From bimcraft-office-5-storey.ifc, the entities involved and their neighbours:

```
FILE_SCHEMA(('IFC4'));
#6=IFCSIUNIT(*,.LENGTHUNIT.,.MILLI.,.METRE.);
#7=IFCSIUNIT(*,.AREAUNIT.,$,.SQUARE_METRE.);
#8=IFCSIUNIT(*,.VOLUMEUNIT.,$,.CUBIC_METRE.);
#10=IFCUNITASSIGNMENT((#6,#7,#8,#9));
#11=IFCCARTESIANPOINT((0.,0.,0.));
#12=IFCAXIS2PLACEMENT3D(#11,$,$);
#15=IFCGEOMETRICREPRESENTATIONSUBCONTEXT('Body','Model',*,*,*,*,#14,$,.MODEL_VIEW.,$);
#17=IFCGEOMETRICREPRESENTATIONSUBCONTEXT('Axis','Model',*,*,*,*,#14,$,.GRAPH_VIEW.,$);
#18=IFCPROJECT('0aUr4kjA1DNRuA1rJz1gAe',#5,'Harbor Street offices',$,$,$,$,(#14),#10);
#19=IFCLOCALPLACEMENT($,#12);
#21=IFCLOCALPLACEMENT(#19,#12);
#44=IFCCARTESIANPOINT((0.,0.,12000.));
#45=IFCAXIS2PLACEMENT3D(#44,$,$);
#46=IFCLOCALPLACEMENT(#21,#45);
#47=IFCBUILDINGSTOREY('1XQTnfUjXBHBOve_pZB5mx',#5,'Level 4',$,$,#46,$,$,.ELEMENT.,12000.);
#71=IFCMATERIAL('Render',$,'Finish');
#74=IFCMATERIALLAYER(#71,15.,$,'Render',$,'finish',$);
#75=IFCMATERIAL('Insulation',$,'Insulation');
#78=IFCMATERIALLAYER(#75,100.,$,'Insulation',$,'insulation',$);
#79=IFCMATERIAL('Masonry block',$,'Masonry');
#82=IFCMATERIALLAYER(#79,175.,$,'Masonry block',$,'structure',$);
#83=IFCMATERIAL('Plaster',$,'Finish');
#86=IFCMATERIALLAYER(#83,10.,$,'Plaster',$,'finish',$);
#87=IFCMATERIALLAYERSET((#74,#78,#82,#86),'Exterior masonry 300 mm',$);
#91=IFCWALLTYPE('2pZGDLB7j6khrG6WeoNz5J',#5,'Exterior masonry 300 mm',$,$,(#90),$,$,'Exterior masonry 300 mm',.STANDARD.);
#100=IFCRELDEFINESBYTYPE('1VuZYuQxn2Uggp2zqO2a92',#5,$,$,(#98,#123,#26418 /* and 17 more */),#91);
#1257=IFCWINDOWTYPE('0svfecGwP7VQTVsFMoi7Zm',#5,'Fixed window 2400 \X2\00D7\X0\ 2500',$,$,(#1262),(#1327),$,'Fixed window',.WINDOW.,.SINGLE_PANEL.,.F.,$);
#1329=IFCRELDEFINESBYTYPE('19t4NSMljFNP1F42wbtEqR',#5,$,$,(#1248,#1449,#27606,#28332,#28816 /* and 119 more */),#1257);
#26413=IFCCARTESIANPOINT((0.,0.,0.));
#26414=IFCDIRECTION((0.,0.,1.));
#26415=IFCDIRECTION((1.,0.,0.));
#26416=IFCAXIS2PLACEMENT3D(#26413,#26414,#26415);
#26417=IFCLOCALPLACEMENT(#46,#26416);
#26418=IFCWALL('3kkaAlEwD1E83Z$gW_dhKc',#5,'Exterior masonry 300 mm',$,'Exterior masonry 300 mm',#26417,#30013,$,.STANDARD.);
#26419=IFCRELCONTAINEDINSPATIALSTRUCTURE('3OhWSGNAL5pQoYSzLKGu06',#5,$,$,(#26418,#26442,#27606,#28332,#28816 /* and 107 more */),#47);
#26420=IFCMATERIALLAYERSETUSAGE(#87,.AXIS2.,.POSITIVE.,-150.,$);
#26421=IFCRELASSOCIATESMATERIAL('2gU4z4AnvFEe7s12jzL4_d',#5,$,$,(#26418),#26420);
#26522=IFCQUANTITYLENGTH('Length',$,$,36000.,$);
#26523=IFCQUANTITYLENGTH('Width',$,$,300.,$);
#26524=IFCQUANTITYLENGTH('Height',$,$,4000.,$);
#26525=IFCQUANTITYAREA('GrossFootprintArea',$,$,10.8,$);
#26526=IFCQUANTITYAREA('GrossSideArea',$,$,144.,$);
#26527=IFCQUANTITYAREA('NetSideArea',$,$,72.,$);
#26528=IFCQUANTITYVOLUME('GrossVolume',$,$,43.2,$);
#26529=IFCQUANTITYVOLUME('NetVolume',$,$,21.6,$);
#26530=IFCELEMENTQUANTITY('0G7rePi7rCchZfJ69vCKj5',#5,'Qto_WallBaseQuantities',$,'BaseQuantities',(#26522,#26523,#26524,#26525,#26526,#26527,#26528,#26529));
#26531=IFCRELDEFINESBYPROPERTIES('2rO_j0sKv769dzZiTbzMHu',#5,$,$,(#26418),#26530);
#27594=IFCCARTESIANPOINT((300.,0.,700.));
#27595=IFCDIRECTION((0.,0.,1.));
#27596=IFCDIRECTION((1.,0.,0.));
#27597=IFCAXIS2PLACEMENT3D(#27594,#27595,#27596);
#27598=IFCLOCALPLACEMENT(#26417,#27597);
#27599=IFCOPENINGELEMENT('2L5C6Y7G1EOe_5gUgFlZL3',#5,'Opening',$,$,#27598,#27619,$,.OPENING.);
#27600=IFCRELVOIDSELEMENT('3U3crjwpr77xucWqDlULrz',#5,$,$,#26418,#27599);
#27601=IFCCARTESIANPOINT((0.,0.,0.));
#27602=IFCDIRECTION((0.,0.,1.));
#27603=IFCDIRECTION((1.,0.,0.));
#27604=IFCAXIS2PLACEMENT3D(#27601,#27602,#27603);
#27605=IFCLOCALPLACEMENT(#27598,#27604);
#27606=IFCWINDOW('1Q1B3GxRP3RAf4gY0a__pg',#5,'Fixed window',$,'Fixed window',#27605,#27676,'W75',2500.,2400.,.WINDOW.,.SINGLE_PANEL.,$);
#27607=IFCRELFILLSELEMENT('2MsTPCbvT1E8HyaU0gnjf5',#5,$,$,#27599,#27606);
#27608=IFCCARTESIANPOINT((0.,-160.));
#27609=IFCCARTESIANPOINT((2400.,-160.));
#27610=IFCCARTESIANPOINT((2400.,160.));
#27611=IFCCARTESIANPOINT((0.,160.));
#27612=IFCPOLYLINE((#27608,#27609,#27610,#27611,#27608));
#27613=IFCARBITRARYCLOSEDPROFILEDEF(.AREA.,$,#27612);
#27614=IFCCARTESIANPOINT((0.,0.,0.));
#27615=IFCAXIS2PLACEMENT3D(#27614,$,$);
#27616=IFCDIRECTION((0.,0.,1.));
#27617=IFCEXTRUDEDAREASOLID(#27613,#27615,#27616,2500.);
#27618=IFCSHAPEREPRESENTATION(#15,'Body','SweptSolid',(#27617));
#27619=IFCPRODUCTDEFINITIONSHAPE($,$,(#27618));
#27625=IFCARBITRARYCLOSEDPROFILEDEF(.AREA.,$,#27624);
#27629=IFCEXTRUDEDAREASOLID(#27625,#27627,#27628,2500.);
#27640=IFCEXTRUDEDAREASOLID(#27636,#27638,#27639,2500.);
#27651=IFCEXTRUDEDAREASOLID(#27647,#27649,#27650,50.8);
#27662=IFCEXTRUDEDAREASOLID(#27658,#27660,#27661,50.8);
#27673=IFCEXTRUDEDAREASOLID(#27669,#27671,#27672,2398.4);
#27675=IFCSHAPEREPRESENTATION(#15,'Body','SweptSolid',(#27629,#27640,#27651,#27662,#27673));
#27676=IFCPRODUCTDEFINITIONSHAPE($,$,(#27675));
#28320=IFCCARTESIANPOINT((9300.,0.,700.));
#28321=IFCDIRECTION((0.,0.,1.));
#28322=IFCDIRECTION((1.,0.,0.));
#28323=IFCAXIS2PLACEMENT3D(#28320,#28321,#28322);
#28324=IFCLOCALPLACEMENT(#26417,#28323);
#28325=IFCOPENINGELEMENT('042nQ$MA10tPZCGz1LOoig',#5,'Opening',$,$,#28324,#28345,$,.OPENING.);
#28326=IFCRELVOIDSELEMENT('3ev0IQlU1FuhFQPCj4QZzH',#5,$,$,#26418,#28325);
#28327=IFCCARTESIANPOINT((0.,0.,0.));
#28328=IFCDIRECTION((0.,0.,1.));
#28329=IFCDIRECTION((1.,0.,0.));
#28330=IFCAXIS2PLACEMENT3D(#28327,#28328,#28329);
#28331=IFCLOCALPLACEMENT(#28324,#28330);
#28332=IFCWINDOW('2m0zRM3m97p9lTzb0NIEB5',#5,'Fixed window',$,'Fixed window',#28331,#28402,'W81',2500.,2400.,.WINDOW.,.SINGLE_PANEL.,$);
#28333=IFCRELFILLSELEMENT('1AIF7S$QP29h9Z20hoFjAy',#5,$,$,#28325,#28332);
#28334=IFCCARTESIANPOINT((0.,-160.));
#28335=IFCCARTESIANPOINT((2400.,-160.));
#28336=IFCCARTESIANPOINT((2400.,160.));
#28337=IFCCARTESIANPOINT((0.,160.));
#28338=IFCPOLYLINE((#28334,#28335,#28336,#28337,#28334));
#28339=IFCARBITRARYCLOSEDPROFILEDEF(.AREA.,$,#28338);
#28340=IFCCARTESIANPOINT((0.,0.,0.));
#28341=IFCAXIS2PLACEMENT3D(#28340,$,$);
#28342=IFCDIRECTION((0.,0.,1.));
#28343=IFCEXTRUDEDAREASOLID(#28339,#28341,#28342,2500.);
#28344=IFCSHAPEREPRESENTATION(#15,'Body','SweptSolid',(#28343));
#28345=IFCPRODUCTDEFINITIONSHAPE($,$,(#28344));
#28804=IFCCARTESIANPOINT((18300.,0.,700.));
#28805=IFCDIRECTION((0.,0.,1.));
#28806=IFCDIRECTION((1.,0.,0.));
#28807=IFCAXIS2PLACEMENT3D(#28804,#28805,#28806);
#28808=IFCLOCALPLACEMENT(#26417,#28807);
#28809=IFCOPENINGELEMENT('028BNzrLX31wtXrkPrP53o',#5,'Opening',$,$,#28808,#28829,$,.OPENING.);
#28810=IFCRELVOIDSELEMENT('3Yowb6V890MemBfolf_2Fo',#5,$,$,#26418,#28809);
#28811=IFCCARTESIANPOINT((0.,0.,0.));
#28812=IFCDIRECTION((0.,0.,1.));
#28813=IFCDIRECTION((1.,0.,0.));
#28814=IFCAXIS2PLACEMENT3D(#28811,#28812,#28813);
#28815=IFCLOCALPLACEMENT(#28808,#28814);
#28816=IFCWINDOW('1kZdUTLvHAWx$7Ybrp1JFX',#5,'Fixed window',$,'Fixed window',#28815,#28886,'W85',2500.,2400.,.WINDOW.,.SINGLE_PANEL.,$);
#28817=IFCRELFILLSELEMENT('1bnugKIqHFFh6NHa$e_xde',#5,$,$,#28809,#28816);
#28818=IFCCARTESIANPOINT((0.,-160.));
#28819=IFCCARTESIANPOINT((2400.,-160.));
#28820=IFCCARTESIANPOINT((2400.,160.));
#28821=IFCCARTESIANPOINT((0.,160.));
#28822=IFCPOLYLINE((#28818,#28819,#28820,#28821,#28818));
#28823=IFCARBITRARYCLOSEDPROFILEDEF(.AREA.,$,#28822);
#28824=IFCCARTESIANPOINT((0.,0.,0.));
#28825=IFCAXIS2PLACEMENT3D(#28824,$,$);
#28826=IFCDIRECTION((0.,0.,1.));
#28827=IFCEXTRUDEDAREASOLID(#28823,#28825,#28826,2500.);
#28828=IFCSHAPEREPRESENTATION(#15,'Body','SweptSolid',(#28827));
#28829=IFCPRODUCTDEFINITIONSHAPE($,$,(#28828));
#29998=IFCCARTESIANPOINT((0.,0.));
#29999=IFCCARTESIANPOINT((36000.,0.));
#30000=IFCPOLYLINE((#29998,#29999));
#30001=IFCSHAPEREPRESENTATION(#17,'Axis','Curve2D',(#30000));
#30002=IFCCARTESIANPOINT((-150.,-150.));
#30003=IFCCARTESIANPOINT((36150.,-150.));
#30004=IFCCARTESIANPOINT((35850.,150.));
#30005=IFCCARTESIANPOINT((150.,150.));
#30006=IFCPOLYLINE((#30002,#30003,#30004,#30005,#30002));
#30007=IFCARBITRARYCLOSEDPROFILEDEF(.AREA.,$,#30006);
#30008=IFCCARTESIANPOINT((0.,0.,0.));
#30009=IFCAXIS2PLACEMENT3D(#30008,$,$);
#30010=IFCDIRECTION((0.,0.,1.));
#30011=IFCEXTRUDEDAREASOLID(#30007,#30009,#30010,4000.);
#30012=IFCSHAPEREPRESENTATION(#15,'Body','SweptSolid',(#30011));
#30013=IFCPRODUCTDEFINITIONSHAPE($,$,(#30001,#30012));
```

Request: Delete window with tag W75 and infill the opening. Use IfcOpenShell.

```python
import ifcopenshell
import ifcopenshell.api.feature
import ifcopenshell.api.pset
import ifcopenshell.api.root
import ifcopenshell.geom
import ifcopenshell.util.element
import ifcopenshell.util.shape
import ifcopenshell.util.unit

model = ifcopenshell.open("bimcraft-office-5-storey.ifc")
area_scale = ifcopenshell.util.unit.calculate_unit_scale(model, "AREAUNIT")
volume_scale = ifcopenshell.util.unit.calculate_unit_scale(model, "VOLUMEUNIT")
settings = ifcopenshell.geom.settings()


def volume(element):
    """Net volume in cubic metres, openings subtracted."""
    shape = ifcopenshell.geom.create_shape(settings, element)
    return ifcopenshell.util.shape.get_volume(shape.geometry)


window = model.by_guid("1Q1B3GxRP3RAf4gY0a__pg")
opening = window.FillsVoids[0].RelatingOpeningElement
wall = opening.VoidsElements[0].RelatingBuildingElement
before = volume(wall)

ifcopenshell.api.root.remove_product(model, product=window)
ifcopenshell.api.feature.remove_feature(model, feature=opening)

after = volume(wall)
thickness = 0.3  # wall thickness in metres

# Update the wall's stored quantities.
qto = model.by_id(ifcopenshell.util.element.get_pset(wall, "Qto_WallBaseQuantities", should_inherit=False)["id"])
ifcopenshell.api.pset.edit_qto(model, qto=qto, properties={
    "NetSideArea": after / thickness / area_scale,
    "NetVolume": after / volume_scale,
})

print(f"wall volume {before:.3f} -> {after:.3f} m3")

model.write("bimcraft-office-5-storey_v2.ifc")
```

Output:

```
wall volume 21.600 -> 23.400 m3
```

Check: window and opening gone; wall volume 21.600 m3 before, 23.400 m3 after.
